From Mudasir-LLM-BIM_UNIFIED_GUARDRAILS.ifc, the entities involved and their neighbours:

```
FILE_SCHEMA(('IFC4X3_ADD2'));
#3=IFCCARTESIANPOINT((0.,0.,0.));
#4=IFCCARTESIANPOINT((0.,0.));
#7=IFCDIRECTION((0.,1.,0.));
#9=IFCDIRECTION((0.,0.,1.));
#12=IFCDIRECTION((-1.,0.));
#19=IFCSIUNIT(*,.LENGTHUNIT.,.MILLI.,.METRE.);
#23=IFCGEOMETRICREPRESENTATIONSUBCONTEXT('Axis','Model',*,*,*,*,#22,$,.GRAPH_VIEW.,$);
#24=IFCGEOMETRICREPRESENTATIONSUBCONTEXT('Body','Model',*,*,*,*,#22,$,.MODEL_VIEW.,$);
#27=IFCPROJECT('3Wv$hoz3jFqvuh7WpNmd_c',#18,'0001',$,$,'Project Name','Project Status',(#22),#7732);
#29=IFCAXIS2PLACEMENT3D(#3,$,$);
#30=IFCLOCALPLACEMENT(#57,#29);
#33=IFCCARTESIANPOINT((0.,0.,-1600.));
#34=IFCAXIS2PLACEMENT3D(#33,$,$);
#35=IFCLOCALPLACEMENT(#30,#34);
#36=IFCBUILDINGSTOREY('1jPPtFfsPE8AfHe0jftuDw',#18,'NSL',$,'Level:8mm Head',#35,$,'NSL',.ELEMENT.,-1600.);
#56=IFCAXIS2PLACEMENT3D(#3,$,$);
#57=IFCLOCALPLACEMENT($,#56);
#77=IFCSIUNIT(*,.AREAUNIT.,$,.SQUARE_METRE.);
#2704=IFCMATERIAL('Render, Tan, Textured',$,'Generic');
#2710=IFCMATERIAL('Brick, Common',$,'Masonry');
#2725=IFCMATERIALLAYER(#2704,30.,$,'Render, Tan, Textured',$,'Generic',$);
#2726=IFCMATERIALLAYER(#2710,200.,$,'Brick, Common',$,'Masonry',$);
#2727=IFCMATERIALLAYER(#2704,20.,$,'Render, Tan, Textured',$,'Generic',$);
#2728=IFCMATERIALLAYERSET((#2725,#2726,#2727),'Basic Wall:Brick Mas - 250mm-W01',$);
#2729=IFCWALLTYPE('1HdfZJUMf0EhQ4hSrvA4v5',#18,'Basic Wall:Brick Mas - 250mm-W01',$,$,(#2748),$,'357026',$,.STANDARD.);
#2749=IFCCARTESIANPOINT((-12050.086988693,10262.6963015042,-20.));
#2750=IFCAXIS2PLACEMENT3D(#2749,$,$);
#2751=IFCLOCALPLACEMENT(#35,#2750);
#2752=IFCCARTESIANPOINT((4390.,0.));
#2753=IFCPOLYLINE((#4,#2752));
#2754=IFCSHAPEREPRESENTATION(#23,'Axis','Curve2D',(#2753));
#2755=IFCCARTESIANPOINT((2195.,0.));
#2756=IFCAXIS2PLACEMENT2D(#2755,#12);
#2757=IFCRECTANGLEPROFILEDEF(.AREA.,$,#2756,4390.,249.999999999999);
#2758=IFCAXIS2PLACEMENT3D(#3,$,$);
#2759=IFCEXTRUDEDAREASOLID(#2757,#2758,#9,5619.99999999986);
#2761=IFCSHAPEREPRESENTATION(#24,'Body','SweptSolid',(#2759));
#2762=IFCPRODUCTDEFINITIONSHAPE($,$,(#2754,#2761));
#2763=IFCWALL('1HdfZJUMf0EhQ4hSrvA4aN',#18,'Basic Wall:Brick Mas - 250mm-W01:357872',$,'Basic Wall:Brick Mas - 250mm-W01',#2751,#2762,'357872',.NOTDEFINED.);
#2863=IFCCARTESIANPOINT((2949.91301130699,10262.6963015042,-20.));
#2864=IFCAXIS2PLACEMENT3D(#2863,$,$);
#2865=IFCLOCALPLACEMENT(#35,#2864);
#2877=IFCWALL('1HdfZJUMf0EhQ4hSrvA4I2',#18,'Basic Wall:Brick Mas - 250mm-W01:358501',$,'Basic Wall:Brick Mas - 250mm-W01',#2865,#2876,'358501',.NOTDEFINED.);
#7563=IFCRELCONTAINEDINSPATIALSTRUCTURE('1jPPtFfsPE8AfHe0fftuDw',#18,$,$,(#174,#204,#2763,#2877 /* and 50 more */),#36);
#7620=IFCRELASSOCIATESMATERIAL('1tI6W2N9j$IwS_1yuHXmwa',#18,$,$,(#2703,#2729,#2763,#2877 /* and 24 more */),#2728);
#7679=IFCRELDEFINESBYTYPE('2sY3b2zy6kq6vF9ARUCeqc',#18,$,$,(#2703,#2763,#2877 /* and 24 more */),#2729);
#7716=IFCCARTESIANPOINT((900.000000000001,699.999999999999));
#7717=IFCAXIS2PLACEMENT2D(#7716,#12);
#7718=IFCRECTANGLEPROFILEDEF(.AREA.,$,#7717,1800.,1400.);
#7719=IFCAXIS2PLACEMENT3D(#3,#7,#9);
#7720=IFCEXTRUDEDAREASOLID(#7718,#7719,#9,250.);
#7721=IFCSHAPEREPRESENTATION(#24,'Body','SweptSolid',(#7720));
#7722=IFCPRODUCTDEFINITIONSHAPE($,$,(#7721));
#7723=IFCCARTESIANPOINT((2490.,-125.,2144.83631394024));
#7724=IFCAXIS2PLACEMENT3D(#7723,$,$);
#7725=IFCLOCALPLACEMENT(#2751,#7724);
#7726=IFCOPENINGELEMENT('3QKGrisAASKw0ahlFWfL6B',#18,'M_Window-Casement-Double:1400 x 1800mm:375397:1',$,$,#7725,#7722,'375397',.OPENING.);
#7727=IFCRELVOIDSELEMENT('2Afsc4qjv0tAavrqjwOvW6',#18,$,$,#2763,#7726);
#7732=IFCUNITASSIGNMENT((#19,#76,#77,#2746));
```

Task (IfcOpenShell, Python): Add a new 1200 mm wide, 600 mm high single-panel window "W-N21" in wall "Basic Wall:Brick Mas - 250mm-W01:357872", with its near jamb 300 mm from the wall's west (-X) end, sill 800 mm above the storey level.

```python
import numpy as np
import ifcopenshell
import ifcopenshell.api.feature
import ifcopenshell.api.geometry
import ifcopenshell.api.root
import ifcopenshell.api.spatial
import ifcopenshell.geom
import ifcopenshell.util.element
import ifcopenshell.util.placement
import ifcopenshell.util.representation
import ifcopenshell.util.shape
import ifcopenshell.util.unit

model = ifcopenshell.open("Mudasir-LLM-BIM_UNIFIED_GUARDRAILS.ifc")
unit_scale = ifcopenshell.util.unit.calculate_unit_scale(model)
settings = ifcopenshell.geom.settings()


def volume(element):
    """Net volume in cubic metres, openings subtracted."""
    shape = ifcopenshell.geom.create_shape(settings, element)
    return ifcopenshell.util.shape.get_volume(shape.geometry)


wall = model.by_id(2763)
storey = ifcopenshell.util.element.get_container(wall, ifc_class="IfcBuildingStorey")
context = ifcopenshell.util.representation.get_context(model, "Model", "Body", "MODEL_VIEW")
before = volume(wall)

width, height, from_end, sill = 1.2, 0.6, 0.3, 0.8  # metres

# The wall runs along its own X axis, and the end named is its -X end.
wall_shape = ifcopenshell.geom.create_shape(settings, wall)
x, y, z = ifcopenshell.util.shape.get_vertices(wall_shape.geometry).T
start = x.min() + from_end
face, thickness = float(y.min()), float(y.max() - y.min())
wall_matrix = ifcopenshell.util.placement.get_local_placement(wall.ObjectPlacement)
level = ifcopenshell.util.placement.get_local_placement(storey.ObjectPlacement)[2, 3]


def in_wall(x, y):
    """Placement at x, y metres in the wall's axes, at sill height."""
    matrix = wall_matrix.copy()
    matrix[:, 3] = wall_matrix @ np.array([x / unit_scale, y / unit_scale, 0.0, 1.0])
    matrix[2, 3] = level + sill / unit_scale
    return matrix


# Opening: a box that overshoots both wall faces by 50 mm.
opening = ifcopenshell.api.root.create_entity(model, ifc_class="IfcOpeningElement", predefined_type="OPENING")
box = ifcopenshell.api.geometry.add_wall_representation(
    model, context=context, length=width, height=height, thickness=thickness + 0.1
)
ifcopenshell.api.geometry.assign_representation(model, product=opening, representation=box)
ifcopenshell.api.geometry.edit_object_placement(model, product=opening, matrix=in_wall(start, face - 0.05), is_si=False)
ifcopenshell.api.feature.add_feature(model, feature=opening, element=wall)

window = ifcopenshell.api.root.create_entity(model, ifc_class="IfcWindow", name="W-N21", predefined_type="WINDOW")
window.OverallWidth, window.OverallHeight = width / unit_scale, height / unit_scale
window.PartitioningType = "SINGLE_PANEL"
body = ifcopenshell.api.geometry.add_window_representation(
    model,
    context=context,
    overall_width=window.OverallWidth,
    overall_height=window.OverallHeight,
    partition_type="SINGLE_PANEL",
)
ifcopenshell.api.geometry.assign_representation(model, product=window, representation=body)
ifcopenshell.api.spatial.assign_container(model, products=[window], relating_structure=storey)
ifcopenshell.api.feature.add_filling(model, opening=opening, element=window)

# Centre the window in the wall's thickness.
ifcopenshell.api.geometry.edit_object_placement(model, product=window, matrix=in_wall(start, face), is_si=False)
window_shape = ifcopenshell.geom.create_shape(settings, window)
depth = ifcopenshell.util.shape.get_vertices(window_shape.geometry)[:, 1]
offset = face + thickness / 2 - (depth.min() + depth.max()) / 2
ifcopenshell.api.geometry.edit_object_placement(model, product=window, matrix=in_wall(start, offset), is_si=False)

after = volume(wall)

print(f"wall volume {before:.3f} -> {after:.3f} m3")

model.write("Mudasir-LLM-BIM_UNIFIED_GUARDRAILS_v2.ifc")
```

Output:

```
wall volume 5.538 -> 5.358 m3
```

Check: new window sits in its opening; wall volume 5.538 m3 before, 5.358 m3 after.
